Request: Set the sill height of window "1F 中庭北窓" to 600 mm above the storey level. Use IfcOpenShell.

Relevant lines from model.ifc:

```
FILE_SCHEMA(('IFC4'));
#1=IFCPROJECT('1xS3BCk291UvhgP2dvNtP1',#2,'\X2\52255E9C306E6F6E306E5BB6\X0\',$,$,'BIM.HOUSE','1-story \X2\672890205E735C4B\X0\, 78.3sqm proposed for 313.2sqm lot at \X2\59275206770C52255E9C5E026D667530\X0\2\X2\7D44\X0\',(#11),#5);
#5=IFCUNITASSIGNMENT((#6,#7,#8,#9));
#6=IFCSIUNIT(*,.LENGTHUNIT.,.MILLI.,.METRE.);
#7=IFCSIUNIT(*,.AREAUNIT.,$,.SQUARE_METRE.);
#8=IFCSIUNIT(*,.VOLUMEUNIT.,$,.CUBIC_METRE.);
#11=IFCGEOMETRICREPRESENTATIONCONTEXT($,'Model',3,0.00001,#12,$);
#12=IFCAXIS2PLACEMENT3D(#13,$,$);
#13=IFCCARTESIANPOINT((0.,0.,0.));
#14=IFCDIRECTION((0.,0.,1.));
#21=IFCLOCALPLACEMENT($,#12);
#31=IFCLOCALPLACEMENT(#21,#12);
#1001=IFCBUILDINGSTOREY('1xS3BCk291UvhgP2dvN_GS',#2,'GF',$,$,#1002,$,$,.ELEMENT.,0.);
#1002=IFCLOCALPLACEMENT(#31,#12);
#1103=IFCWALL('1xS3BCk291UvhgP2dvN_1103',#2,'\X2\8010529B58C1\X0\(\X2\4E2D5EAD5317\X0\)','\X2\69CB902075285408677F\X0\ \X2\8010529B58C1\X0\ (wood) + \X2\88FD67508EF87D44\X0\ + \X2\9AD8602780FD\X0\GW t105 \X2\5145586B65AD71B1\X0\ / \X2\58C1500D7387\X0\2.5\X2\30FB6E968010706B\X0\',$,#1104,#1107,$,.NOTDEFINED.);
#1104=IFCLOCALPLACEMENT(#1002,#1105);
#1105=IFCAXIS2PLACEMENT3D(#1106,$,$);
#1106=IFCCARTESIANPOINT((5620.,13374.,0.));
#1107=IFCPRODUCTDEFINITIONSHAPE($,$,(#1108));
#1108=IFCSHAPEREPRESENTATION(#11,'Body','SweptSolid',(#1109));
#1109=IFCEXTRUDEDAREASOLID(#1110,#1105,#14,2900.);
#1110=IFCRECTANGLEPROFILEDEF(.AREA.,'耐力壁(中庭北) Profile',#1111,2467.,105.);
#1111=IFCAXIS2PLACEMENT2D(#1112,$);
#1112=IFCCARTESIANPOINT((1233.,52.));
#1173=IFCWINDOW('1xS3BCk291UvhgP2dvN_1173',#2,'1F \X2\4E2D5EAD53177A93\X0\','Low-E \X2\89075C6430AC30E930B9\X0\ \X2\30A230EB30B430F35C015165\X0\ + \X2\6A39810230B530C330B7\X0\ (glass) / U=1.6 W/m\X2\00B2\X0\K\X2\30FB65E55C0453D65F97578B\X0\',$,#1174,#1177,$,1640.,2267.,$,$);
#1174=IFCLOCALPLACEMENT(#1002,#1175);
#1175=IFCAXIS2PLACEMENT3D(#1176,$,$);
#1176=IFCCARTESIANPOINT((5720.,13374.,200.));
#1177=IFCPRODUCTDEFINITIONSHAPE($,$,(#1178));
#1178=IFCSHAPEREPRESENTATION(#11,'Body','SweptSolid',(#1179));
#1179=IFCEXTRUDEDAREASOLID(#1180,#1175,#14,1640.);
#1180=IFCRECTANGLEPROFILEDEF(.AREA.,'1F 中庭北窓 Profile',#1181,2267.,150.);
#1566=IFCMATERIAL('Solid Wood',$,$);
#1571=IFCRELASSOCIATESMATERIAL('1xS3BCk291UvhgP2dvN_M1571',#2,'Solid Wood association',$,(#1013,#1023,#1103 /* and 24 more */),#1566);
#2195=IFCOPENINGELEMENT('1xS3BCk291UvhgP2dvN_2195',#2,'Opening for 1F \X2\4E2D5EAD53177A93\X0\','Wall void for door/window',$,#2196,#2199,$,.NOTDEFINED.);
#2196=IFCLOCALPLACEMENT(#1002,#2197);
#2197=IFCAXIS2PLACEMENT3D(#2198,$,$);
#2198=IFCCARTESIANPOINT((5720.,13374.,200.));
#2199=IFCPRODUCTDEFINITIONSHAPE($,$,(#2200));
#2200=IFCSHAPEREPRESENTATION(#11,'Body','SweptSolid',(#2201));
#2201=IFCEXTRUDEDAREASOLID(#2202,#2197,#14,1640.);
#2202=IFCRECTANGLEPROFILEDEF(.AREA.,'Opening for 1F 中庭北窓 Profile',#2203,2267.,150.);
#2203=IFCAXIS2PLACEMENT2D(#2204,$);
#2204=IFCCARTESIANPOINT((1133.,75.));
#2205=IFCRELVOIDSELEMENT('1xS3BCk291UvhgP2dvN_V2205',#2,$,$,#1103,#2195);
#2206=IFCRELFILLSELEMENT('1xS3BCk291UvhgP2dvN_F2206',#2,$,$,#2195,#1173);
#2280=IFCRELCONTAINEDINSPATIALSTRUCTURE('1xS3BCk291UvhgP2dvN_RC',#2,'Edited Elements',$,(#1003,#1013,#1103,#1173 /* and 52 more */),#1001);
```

```python
import numpy as np
import ifcopenshell
import ifcopenshell.api.geometry
import ifcopenshell.geom
import ifcopenshell.util.element
import ifcopenshell.util.placement
import ifcopenshell.util.shape
import ifcopenshell.util.unit

model = ifcopenshell.open("model.ifc")
unit_scale = ifcopenshell.util.unit.calculate_unit_scale(model)

window = model.by_guid("1xS3BCk291UvhgP2dvN_1173")
opening = window.FillsVoids[0].RelatingOpeningElement
storey = ifcopenshell.util.element.get_container(window, ifc_class="IfcBuildingStorey")
level = ifcopenshell.util.placement.get_local_placement(storey.ObjectPlacement)[2, 3]

# The opening's origin need not be at the sill, so measure its lowest point.
shape = ifcopenshell.geom.create_shape(ifcopenshell.geom.settings(), opening)
bottom = ifcopenshell.util.shape.get_shape_bottom_elevation(shape, shape.geometry) / unit_scale
dz = level + 600.0 - bottom

shift = np.array([0.0, 0.0, dz])
# The window is not placed relative to its opening, so move both.
for product in (opening, window):
    matrix = ifcopenshell.util.placement.get_local_placement(product.ObjectPlacement)
    matrix[:3, 3] += shift
    ifcopenshell.api.geometry.edit_object_placement(model, product=product, matrix=matrix, is_si=False)

print(f"moved by {dz * unit_scale:+.3f} m")

model.write("model_updated.ifc")
```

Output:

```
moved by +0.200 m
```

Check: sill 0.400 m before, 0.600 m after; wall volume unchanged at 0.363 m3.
